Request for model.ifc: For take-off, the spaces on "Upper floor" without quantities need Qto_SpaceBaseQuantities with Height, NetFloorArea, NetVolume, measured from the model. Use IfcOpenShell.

First a look at what the model holds.

```python
import ifcopenshell
import ifcopenshell.util.element
import ifcopenshell.util.unit

model = ifcopenshell.open("model.ifc")
print(model.schema)
for unit_type in ("LENGTHUNIT", "AREAUNIT", "VOLUMEUNIT"):
    print(unit_type, ifcopenshell.util.unit.calculate_unit_scale(model, unit_type))
storey = next(s for s in model.by_type("IfcBuildingStorey") if s.Name == "Upper floor")
spaces = [e for e in ifcopenshell.util.element.get_decomposition(storey) if e.is_a("IfcSpace")]
for e in sorted(spaces, key=lambda e: e.id()):
    print(e.id(), e.is_a(), e.Name, list(ifcopenshell.util.element.get_psets(e, qtos_only=True)), sep=" | ")
```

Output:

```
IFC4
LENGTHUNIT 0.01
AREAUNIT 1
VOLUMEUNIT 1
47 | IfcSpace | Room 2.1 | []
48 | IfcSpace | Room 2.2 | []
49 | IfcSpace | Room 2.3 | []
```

```python
import ifcopenshell
import ifcopenshell.api.pset
import ifcopenshell.geom
import ifcopenshell.util.element
import ifcopenshell.util.shape
import ifcopenshell.util.unit

model = ifcopenshell.open("model.ifc")
unit_scale = ifcopenshell.util.unit.calculate_unit_scale(model)
area_scale = ifcopenshell.util.unit.calculate_unit_scale(model, "AREAUNIT")
volume_scale = ifcopenshell.util.unit.calculate_unit_scale(model, "VOLUMEUNIT")
settings = ifcopenshell.geom.settings()

storey = next(s for s in model.by_type("IfcBuildingStorey") if s.Name == "Upper floor")
spaces = [e for e in ifcopenshell.util.element.get_decomposition(storey) if e.is_a("IfcSpace")]

for e in sorted(spaces, key=lambda e: e.id()):
    if ifcopenshell.util.element.get_psets(e, qtos_only=True, should_inherit=False):
        continue
    # Geometry comes back in metres, in the element's own axes.
    shape = ifcopenshell.geom.create_shape(settings, e)
    values = {
        "Height": ifcopenshell.util.shape.get_z(shape.geometry) / unit_scale,
        "NetFloorArea": ifcopenshell.util.shape.get_footprint_area(shape.geometry) / area_scale,
        "NetVolume": ifcopenshell.util.shape.get_volume(shape.geometry) / volume_scale,
    }
    qto = ifcopenshell.api.pset.add_qto(model, product=e, name="Qto_SpaceBaseQuantities")
    ifcopenshell.api.pset.edit_qto(model, qto=qto, properties=values)
    print(e.id(), {k: round(v, 3) for k, v in values.items()})

model.write("model-out.ifc")
```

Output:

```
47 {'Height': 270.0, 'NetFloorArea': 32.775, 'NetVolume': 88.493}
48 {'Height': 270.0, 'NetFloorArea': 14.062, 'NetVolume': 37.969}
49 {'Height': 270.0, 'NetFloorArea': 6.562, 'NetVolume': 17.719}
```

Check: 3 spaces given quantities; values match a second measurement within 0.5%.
